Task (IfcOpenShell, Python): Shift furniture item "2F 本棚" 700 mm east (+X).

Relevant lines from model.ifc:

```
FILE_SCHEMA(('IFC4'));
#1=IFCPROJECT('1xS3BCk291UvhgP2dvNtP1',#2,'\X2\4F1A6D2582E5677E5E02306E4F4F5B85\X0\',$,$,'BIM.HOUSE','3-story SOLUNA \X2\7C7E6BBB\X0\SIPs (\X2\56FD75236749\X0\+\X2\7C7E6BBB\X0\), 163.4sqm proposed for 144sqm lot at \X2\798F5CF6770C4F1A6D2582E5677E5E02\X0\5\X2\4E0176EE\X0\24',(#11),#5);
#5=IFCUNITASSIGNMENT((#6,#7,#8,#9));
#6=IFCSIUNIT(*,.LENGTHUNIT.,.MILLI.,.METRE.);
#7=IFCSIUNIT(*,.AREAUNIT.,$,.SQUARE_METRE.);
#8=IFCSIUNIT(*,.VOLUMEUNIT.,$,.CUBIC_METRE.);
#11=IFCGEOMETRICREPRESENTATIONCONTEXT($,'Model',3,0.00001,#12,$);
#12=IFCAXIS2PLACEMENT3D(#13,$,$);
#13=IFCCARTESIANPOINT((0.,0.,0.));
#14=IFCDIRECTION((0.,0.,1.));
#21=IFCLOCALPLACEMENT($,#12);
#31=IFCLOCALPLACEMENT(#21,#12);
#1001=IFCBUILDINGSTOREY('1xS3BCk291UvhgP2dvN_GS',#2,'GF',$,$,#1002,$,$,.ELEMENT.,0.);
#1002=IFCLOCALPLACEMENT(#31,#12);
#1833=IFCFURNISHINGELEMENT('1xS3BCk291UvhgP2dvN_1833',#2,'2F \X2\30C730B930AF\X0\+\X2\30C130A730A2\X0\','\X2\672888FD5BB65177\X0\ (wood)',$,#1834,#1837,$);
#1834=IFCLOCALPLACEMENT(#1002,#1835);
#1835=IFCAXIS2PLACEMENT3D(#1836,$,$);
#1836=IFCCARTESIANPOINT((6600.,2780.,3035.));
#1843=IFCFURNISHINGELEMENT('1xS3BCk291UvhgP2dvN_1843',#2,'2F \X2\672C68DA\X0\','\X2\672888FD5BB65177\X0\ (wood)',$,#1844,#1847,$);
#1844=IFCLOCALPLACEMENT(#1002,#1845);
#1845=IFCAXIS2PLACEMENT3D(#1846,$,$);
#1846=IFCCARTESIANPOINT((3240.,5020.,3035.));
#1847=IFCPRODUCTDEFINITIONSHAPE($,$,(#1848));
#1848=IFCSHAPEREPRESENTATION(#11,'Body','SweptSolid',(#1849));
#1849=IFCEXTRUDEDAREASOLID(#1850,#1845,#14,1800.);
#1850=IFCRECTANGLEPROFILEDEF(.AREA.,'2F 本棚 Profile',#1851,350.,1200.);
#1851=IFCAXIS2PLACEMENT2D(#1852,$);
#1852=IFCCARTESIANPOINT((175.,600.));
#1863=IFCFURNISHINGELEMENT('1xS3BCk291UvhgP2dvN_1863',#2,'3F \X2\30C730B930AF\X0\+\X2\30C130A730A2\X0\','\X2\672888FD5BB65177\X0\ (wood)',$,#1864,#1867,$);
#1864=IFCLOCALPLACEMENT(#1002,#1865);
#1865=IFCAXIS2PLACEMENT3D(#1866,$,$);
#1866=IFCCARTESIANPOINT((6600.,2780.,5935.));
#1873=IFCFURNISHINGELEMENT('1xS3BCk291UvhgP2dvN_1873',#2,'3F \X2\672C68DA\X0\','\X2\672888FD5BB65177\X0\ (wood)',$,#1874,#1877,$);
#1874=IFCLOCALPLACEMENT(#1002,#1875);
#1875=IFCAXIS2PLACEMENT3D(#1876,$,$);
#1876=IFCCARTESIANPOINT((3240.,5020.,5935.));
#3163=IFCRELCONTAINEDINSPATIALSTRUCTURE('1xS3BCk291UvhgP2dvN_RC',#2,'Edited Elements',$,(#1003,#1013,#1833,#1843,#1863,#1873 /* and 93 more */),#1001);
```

```python
import ifcopenshell
import ifcopenshell.api.geometry
import ifcopenshell.util.placement
import ifcopenshell.util.unit

model = ifcopenshell.open("model.ifc")
unit_scale = ifcopenshell.util.unit.calculate_unit_scale(model)

item = model.by_guid("1xS3BCk291UvhgP2dvN_1843")
matrix = ifcopenshell.util.placement.get_local_placement(item.ObjectPlacement)
matrix[0, 3] += 0.7 / unit_scale
ifcopenshell.api.geometry.edit_object_placement(model, product=item, matrix=matrix, is_si=False)

print(ifcopenshell.util.placement.get_local_placement(item.ObjectPlacement).round(3) + 0.0)

model.write("model_edited.ifc")
```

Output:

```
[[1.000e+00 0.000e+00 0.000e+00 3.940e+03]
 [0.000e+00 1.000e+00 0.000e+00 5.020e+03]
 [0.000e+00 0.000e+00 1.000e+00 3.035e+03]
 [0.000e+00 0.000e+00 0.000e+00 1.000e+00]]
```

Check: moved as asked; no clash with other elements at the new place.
